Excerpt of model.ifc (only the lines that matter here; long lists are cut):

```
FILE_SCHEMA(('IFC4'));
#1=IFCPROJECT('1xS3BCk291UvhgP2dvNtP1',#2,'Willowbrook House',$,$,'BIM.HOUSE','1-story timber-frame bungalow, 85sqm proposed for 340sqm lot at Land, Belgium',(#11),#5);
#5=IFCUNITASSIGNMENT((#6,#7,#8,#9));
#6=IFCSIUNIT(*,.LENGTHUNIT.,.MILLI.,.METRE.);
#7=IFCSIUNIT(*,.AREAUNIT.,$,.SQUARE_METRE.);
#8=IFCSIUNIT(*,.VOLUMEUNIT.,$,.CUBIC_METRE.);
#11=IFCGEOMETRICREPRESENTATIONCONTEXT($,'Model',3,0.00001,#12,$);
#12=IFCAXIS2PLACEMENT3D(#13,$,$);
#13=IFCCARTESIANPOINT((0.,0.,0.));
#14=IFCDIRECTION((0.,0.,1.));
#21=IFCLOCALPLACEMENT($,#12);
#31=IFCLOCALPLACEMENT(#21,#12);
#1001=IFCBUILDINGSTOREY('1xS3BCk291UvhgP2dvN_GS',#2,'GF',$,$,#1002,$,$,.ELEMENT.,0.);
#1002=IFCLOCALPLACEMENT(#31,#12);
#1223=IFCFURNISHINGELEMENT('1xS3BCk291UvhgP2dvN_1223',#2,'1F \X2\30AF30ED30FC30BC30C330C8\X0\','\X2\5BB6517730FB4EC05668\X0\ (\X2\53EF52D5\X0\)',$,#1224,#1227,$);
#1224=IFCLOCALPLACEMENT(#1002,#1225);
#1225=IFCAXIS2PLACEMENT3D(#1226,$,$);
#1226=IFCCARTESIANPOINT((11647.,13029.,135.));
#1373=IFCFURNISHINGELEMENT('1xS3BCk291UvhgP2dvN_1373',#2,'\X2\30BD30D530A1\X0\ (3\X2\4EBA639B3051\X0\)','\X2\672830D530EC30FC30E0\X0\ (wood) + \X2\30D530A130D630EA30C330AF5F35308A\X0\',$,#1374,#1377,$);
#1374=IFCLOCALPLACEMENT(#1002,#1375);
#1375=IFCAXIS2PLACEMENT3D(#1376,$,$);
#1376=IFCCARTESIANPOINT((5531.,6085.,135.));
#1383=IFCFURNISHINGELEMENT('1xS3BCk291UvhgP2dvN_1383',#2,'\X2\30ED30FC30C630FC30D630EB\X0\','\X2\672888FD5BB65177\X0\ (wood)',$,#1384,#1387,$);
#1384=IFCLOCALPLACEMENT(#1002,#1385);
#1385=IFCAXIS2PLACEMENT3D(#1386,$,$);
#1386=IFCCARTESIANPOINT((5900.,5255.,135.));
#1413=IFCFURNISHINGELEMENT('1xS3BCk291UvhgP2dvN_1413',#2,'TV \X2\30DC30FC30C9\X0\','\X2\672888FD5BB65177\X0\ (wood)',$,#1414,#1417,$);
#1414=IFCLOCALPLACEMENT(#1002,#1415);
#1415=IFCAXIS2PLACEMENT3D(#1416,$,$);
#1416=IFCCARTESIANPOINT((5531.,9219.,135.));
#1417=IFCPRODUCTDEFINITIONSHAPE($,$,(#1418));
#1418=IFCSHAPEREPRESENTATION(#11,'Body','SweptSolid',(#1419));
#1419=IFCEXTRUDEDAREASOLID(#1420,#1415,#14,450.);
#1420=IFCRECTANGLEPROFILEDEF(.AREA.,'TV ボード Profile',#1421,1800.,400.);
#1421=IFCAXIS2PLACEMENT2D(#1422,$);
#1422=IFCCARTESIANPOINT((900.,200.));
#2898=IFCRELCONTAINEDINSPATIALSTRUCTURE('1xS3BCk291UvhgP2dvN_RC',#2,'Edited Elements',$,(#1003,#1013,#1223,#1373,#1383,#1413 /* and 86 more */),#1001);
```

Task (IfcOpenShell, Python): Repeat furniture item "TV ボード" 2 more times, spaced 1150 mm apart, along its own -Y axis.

```python
import ifcopenshell
import ifcopenshell.api.geometry
import ifcopenshell.api.root
import ifcopenshell.util.element
import ifcopenshell.util.placement
import ifcopenshell.util.unit

model = ifcopenshell.open("model.ifc")
unit_scale = ifcopenshell.util.unit.calculate_unit_scale(model)


def reuse_history(source, copy):
    """copy_class also copies each property set's owner history, people and application; keep the originals."""
    for rel in copy.IsDefinedBy:
        if rel.is_a("IfcRelDefinesByProperties") and (history := rel.RelatingPropertyDefinition.OwnerHistory):
            rel.RelatingPropertyDefinition.OwnerHistory = source.OwnerHistory
            ifcopenshell.util.element.remove_deep2(model, history)


source = model.by_guid("1xS3BCk291UvhgP2dvN_1413")
base = ifcopenshell.util.placement.get_local_placement(source.ObjectPlacement)
step = -base[:3, 1] * 1.15 / unit_scale

for i in range(1, 3):
    copy = ifcopenshell.api.root.copy_class(model, product=source)
    copy.Representation = ifcopenshell.util.element.copy_deep(
        model, source.Representation, exclude=["IfcGeometricRepresentationContext", "IfcRepresentationMap"]
    )
    reuse_history(source, copy)
    matrix = base.copy()
    matrix[:3, 3] += i * step
    print("added at", matrix[:3, 3].round(3) + 0.0)
    ifcopenshell.api.geometry.edit_object_placement(model, product=copy, matrix=matrix, is_si=False)

model.write("model_edited.ifc")
```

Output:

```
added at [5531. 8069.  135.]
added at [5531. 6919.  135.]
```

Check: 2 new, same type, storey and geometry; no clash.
